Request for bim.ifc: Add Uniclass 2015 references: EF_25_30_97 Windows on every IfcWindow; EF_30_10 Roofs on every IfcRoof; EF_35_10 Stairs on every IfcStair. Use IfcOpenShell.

First a look at what the model holds.

```python
import ifcopenshell

model = ifcopenshell.open("bim.ifc")
print(model.schema)
print("classifications:", [c.Name for c in model.by_type("IfcClassification")])
for ifc_class in ("IfcDoor", "IfcRoof", "IfcStair", "IfcWall", "IfcWindow"):
    print(ifc_class, len(model.by_type(ifc_class)))
```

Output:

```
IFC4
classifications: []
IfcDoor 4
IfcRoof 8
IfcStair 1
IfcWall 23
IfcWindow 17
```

```python
import ifcopenshell
import ifcopenshell.api.classification

model = ifcopenshell.open("bim.ifc")

system = ifcopenshell.api.classification.add_classification(model, classification="Uniclass 2015")

codes = {
    "IfcWindow": ("EF_25_30_97", "Windows"),
    "IfcRoof": ("EF_30_10", "Roofs"),
    "IfcStair": ("EF_35_10", "Stairs"),
}
for ifc_class, (code, name) in codes.items():
    products = model.by_type(ifc_class)
    ifcopenshell.api.classification.add_reference(
        model, products=products, classification=system, identification=code, name=name
    )
    print(code, len(products))

model.write("bim_edited.ifc")
```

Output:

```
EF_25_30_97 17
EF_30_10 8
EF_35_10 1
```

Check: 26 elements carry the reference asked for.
